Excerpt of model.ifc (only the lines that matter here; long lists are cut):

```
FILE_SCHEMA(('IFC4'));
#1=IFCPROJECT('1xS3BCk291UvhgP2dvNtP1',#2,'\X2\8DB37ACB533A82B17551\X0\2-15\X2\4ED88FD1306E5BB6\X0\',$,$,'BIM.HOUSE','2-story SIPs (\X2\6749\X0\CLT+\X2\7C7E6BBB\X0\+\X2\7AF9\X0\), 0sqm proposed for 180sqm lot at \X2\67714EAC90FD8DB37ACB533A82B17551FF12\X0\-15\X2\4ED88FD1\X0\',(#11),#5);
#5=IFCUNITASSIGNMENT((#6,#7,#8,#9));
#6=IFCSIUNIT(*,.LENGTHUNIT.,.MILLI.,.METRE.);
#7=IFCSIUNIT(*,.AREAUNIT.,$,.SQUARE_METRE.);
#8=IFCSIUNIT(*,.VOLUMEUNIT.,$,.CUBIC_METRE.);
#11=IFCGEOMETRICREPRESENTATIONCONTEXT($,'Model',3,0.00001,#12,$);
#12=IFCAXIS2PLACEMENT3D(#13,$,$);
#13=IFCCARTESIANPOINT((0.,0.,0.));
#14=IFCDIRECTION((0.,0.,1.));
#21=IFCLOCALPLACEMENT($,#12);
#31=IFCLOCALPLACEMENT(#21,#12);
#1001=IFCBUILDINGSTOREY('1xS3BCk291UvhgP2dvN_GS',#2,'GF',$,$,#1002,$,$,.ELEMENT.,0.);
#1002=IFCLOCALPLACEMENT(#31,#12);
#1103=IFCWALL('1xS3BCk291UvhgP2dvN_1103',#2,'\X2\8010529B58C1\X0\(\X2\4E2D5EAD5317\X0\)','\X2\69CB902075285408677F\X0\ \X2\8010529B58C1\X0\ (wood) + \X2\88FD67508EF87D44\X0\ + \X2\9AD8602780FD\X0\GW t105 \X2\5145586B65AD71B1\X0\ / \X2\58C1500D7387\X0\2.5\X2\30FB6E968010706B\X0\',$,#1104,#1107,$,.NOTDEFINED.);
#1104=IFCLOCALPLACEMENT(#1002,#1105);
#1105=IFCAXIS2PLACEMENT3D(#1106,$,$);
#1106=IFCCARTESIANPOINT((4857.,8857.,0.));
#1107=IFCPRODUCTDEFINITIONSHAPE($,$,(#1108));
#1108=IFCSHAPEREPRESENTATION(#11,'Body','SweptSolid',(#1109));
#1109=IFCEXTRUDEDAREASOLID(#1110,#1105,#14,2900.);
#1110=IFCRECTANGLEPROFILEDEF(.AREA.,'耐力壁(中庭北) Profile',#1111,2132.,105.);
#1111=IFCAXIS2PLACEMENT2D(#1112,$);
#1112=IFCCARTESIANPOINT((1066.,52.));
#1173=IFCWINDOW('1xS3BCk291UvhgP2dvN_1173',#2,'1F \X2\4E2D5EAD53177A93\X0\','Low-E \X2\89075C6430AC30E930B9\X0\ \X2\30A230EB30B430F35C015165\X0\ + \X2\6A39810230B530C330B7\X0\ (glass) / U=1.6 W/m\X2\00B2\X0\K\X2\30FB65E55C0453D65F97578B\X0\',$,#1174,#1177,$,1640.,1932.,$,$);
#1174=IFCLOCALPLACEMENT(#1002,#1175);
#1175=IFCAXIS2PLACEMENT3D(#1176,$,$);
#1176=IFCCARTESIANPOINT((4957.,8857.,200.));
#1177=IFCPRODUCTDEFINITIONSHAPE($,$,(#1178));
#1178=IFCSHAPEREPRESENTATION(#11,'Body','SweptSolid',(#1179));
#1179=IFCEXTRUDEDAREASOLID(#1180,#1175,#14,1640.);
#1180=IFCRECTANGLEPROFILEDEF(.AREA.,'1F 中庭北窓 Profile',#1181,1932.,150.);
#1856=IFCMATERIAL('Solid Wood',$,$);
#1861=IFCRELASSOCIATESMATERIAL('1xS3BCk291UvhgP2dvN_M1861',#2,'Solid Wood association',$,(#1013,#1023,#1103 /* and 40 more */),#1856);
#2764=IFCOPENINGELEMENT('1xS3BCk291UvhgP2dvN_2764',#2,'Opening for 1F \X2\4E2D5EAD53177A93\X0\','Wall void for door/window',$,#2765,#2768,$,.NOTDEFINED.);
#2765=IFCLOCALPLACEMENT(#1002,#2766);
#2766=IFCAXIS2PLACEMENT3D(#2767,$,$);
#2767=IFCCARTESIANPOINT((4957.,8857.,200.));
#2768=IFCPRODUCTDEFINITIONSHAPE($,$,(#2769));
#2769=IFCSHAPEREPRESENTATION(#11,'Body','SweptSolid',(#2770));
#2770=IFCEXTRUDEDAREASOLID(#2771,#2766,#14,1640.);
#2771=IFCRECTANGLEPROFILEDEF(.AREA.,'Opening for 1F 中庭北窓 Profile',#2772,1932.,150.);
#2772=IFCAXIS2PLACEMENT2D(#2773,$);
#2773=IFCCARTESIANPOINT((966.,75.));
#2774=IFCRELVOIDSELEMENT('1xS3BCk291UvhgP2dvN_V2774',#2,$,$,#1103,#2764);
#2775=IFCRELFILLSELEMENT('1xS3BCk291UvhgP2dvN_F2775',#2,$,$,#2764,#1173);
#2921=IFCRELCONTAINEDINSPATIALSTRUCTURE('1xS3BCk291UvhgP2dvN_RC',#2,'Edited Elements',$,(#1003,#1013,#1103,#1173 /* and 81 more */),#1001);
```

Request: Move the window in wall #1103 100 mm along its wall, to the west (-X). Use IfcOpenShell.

```python
import ifcopenshell
import ifcopenshell.api.geometry
import ifcopenshell.util.placement

model = ifcopenshell.open("model.ifc")

window = model.by_guid("1xS3BCk291UvhgP2dvN_1173")
opening = window.FillsVoids[0].RelatingOpeningElement
wall = opening.VoidsElements[0].RelatingBuildingElement

wall_matrix = ifcopenshell.util.placement.get_local_placement(wall.ObjectPlacement)
shift = wall_matrix[:3, 0] * -100.0
before = ifcopenshell.util.placement.get_local_placement(window.ObjectPlacement)[:3, 3].copy()

# The window is not placed relative to its opening, so move both.
for product in (opening, window):
    matrix = ifcopenshell.util.placement.get_local_placement(product.ObjectPlacement)
    matrix[:3, 3] += shift
    ifcopenshell.api.geometry.edit_object_placement(model, product=product, matrix=matrix, is_si=False)

after = ifcopenshell.util.placement.get_local_placement(window.ObjectPlacement)[:3, 3]
print("window moved by", (after - before).round(3) + 0.0)

model.write("model-out.ifc")
```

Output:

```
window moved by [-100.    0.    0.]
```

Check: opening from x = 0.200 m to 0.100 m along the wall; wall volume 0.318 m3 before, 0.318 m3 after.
